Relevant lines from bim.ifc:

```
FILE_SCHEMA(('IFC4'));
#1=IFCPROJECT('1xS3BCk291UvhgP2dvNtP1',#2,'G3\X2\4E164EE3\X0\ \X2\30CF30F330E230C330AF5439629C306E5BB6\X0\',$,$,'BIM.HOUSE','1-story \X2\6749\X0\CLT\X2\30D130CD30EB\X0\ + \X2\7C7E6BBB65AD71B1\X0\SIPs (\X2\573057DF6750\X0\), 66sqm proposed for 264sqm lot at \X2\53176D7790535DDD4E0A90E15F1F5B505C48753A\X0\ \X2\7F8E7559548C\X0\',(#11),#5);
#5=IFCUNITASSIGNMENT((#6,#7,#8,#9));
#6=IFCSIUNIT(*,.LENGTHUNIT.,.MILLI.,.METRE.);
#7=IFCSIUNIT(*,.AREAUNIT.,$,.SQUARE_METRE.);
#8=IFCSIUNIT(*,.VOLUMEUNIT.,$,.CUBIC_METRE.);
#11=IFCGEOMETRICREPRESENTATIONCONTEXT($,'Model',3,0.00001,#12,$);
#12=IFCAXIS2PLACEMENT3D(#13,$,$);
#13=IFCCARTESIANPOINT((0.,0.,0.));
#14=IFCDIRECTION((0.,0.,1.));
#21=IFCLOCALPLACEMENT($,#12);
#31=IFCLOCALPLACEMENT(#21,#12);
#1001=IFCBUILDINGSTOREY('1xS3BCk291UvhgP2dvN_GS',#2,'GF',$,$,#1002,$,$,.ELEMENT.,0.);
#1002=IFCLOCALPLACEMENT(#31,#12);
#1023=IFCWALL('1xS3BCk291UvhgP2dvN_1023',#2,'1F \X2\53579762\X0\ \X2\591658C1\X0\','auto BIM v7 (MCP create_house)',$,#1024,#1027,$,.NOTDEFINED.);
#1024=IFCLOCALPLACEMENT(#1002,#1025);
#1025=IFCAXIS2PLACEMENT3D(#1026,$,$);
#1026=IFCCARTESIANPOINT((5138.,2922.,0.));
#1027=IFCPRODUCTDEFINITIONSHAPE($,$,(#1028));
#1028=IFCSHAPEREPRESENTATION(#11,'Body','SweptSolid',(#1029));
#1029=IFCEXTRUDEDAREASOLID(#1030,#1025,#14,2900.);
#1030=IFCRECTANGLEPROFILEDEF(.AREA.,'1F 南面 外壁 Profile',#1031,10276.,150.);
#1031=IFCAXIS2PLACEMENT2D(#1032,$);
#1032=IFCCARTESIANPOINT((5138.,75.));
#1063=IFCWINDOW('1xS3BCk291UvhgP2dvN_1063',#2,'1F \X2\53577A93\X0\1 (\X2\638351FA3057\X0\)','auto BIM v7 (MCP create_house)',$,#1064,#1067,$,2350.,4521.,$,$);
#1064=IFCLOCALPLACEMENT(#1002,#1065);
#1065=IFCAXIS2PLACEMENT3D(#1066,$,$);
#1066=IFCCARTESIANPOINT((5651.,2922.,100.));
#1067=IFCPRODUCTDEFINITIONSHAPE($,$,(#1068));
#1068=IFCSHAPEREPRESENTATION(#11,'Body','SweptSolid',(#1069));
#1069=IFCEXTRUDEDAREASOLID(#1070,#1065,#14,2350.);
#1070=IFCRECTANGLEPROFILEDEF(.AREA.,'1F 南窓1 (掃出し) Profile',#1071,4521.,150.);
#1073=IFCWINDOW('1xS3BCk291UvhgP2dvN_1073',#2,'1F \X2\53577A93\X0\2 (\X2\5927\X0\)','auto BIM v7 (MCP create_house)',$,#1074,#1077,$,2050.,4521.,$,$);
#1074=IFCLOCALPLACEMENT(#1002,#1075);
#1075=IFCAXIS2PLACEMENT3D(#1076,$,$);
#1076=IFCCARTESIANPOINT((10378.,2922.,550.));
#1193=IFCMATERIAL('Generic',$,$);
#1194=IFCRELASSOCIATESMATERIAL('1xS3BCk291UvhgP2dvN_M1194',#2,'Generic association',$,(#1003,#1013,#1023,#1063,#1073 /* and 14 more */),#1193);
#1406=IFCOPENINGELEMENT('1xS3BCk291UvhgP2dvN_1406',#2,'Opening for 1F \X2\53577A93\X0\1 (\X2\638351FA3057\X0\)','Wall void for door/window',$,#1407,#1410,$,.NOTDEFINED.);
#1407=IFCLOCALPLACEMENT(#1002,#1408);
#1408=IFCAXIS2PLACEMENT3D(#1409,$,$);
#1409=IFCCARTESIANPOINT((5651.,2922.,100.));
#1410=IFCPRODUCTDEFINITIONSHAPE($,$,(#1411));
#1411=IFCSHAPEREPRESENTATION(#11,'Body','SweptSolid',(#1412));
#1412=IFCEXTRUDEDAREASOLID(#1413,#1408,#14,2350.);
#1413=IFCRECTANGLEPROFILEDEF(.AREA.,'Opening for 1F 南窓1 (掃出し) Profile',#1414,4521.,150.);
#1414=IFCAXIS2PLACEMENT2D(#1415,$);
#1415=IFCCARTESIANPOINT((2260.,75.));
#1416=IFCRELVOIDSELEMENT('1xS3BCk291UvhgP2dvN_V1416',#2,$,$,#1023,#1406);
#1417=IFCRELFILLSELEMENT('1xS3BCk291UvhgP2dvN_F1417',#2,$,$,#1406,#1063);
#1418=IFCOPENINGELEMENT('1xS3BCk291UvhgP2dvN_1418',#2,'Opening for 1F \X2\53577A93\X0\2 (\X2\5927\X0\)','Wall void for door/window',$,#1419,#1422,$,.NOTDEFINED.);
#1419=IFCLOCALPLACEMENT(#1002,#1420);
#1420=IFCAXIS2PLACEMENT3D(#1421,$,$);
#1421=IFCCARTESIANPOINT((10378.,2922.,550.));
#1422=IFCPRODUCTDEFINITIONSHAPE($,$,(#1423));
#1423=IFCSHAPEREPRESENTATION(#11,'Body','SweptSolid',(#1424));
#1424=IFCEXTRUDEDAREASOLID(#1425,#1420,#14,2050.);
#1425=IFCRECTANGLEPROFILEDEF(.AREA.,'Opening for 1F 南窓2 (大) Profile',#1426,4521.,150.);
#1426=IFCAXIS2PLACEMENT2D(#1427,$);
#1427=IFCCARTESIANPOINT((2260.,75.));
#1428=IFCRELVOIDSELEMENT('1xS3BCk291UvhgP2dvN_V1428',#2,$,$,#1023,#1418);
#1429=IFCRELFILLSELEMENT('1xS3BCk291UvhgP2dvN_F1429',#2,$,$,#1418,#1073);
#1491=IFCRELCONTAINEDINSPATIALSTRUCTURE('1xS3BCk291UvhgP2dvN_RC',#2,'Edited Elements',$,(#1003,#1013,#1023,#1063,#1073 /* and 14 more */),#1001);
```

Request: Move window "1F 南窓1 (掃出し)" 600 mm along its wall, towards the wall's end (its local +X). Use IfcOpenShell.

```python
import ifcopenshell
import ifcopenshell.api.geometry
import ifcopenshell.util.placement
import ifcopenshell.util.unit

model = ifcopenshell.open("bim.ifc")
unit_scale = ifcopenshell.util.unit.calculate_unit_scale(model)

window = model.by_guid("1xS3BCk291UvhgP2dvN_1063")
opening = window.FillsVoids[0].RelatingOpeningElement
wall = opening.VoidsElements[0].RelatingBuildingElement

wall_matrix = ifcopenshell.util.placement.get_local_placement(wall.ObjectPlacement)
shift = wall_matrix[:3, 0] * 0.6 / unit_scale
before = ifcopenshell.util.placement.get_local_placement(window.ObjectPlacement)[:3, 3].copy()

# The window is not placed relative to its opening, so move both.
for product in (opening, window):
    matrix = ifcopenshell.util.placement.get_local_placement(product.ObjectPlacement)
    matrix[:3, 3] += shift
    ifcopenshell.api.geometry.edit_object_placement(model, product=product, matrix=matrix, is_si=False)

after = ifcopenshell.util.placement.get_local_placement(window.ObjectPlacement)[:3, 3]
print("window moved by", (after - before).round(3) + 0.0)

model.write("bim_rev.ifc")
```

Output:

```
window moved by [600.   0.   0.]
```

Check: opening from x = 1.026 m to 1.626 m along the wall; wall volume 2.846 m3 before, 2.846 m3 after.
